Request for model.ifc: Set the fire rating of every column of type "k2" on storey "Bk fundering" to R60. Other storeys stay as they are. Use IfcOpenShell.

First a look at what the model holds.

```python
import ifcopenshell
import ifcopenshell.util.element

model = ifcopenshell.open("model.ifc")
print(model.schema)
storey = next(s for s in model.by_type("IfcBuildingStorey") if s.Name == "Bk fundering")
columns = [e for e in ifcopenshell.util.element.get_decomposition(storey) if e.is_a("IfcColumn")]
seen = {}
for e in columns:
    element_type = ifcopenshell.util.element.get_type(e)
    key = (element_type.Name if element_type != e and element_type else None, ifcopenshell.util.element.get_pset(e, "Pset_ColumnCommon", "FireRating"))
    seen[key] = seen.get(key, 0) + 1
for (name, value), count in sorted(seen.items(), key=str):
    print(count, "x", name, "|", value)
```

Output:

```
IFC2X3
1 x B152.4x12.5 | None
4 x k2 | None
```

```python
import ifcopenshell
import ifcopenshell.api.pset
import ifcopenshell.util.element

model = ifcopenshell.open("model.ifc")

storey = next(s for s in model.by_type("IfcBuildingStorey") if s.Name == "Bk fundering")
columns = [e for e in ifcopenshell.util.element.get_decomposition(storey) if e.is_a("IfcColumn")]

count = 0
for e in columns:
    element_type = ifcopenshell.util.element.get_type(e)
    if element_type in (None, e) or element_type.Name != "k2":
        continue
    # add_pset returns the element's existing set when there is one.
    pset = ifcopenshell.api.pset.add_pset(model, product=e, name="Pset_ColumnCommon")
    ifcopenshell.api.pset.edit_pset(model, pset=pset, properties={"FireRating": "R60"})
    count += 1

print(count, "columns updated")

model.write("model_v2.ifc")
```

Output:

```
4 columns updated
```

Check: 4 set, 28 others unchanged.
